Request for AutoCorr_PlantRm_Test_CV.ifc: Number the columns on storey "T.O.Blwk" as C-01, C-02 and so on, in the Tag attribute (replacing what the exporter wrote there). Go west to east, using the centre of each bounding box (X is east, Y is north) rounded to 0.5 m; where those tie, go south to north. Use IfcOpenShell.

First a look at what the model holds.

```python
import ifcopenshell
import ifcopenshell.util.element
import ifcopenshell.util.placement

model = ifcopenshell.open("AutoCorr_PlantRm_Test_CV.ifc")
print(model.schema)
storey = next(s for s in model.by_type("IfcBuildingStorey") if s.Name == "T.O.Blwk")
columns = [e for e in ifcopenshell.util.element.get_decomposition(storey) if e.is_a("IfcColumn")]
for e in sorted(columns, key=lambda e: e.id()):
    origin = ifcopenshell.util.placement.get_local_placement(e.ObjectPlacement)[:3, 3]
    print(e.id(), e.Tag, e.Name, origin.round(2) + 0.0, sep=" | ")
```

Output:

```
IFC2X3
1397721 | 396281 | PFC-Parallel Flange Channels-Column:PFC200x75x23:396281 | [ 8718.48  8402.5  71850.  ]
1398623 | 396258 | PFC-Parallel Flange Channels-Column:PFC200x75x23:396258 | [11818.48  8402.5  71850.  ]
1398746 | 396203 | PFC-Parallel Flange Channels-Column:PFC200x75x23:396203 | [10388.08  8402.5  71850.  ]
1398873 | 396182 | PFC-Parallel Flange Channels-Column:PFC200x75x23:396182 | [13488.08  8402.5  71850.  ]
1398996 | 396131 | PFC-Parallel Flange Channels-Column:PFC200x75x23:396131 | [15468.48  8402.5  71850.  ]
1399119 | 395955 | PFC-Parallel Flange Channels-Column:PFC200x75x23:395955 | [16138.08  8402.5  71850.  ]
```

```python
import ifcopenshell
import ifcopenshell.geom
import ifcopenshell.util.element
import ifcopenshell.util.shape

model = ifcopenshell.open("AutoCorr_PlantRm_Test_CV.ifc")
settings = ifcopenshell.geom.settings()
settings.set("use-world-coords", True)


def centre(element):
    shape = ifcopenshell.geom.create_shape(settings, element)
    return ifcopenshell.util.shape.get_bbox_centroid(shape.geometry)


storey = next(s for s in model.by_type("IfcBuildingStorey") if s.Name == "T.O.Blwk")
columns = [e for e in ifcopenshell.util.element.get_decomposition(storey) if e.is_a("IfcColumn")]

# Insertion points can sit at a corner or the storey origin, so sort by the geometry (in metres).
centres = {e: centre(e) for e in columns}
columns.sort(key=lambda e: (round(centres[e][0] / 0.5), centres[e][1]))

for i, e in enumerate(columns, start=1):
    number = f"C-{i:02d}"
    e.Tag = number
    print(e.id(), number)

model.write("AutoCorr_PlantRm_Test_CV_updated.ifc")
```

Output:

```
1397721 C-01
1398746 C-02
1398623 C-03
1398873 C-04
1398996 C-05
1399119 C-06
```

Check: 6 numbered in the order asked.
